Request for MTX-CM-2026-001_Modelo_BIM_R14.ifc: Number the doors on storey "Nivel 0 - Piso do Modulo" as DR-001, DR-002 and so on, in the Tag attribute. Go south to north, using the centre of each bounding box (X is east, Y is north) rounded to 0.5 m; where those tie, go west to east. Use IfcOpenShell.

First a look at what the model holds.

```python
import ifcopenshell
import ifcopenshell.util.element
import ifcopenshell.util.placement

model = ifcopenshell.open("MTX-CM-2026-001_Modelo_BIM_R14.ifc")
print(model.schema)
storey = next(s for s in model.by_type("IfcBuildingStorey") if s.Name == "Nivel 0 - Piso do Modulo")
doors = [e for e in ifcopenshell.util.element.get_decomposition(storey) if e.is_a("IfcDoor")]
for e in sorted(doors, key=lambda e: e.id()):
    origin = ifcopenshell.util.placement.get_local_placement(e.ObjectPlacement)[:3, 3]
    print(e.id(), e.Tag, e.Name, origin.round(2) + 0.0, sep=" | ")
```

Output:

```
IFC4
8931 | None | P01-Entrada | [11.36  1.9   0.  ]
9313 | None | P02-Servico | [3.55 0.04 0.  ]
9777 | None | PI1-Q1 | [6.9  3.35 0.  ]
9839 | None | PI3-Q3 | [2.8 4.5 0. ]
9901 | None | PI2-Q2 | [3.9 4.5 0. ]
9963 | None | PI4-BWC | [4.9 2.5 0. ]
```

```python
import ifcopenshell
import ifcopenshell.geom
import ifcopenshell.util.element
import ifcopenshell.util.shape

model = ifcopenshell.open("MTX-CM-2026-001_Modelo_BIM_R14.ifc")
settings = ifcopenshell.geom.settings()
settings.set("use-world-coords", True)


def centre(element):
    shape = ifcopenshell.geom.create_shape(settings, element)
    return ifcopenshell.util.shape.get_bbox_centroid(shape.geometry)


storey = next(s for s in model.by_type("IfcBuildingStorey") if s.Name == "Nivel 0 - Piso do Modulo")
doors = [e for e in ifcopenshell.util.element.get_decomposition(storey) if e.is_a("IfcDoor")]

# Insertion points can sit at a corner or the storey origin, so sort by the geometry (in metres).
centres = {e: centre(e) for e in doors}
doors.sort(key=lambda e: (round(centres[e][1] / 0.5), centres[e][0]))

for i, e in enumerate(doors, start=1):
    number = f"DR-0{i:02d}"
    e.Tag = number
    print(e.id(), number)

model.write("MTX-CM-2026-001_Modelo_BIM_R14_rev.ifc")
```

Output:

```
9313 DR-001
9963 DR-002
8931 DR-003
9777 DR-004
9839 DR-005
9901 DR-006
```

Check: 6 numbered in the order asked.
